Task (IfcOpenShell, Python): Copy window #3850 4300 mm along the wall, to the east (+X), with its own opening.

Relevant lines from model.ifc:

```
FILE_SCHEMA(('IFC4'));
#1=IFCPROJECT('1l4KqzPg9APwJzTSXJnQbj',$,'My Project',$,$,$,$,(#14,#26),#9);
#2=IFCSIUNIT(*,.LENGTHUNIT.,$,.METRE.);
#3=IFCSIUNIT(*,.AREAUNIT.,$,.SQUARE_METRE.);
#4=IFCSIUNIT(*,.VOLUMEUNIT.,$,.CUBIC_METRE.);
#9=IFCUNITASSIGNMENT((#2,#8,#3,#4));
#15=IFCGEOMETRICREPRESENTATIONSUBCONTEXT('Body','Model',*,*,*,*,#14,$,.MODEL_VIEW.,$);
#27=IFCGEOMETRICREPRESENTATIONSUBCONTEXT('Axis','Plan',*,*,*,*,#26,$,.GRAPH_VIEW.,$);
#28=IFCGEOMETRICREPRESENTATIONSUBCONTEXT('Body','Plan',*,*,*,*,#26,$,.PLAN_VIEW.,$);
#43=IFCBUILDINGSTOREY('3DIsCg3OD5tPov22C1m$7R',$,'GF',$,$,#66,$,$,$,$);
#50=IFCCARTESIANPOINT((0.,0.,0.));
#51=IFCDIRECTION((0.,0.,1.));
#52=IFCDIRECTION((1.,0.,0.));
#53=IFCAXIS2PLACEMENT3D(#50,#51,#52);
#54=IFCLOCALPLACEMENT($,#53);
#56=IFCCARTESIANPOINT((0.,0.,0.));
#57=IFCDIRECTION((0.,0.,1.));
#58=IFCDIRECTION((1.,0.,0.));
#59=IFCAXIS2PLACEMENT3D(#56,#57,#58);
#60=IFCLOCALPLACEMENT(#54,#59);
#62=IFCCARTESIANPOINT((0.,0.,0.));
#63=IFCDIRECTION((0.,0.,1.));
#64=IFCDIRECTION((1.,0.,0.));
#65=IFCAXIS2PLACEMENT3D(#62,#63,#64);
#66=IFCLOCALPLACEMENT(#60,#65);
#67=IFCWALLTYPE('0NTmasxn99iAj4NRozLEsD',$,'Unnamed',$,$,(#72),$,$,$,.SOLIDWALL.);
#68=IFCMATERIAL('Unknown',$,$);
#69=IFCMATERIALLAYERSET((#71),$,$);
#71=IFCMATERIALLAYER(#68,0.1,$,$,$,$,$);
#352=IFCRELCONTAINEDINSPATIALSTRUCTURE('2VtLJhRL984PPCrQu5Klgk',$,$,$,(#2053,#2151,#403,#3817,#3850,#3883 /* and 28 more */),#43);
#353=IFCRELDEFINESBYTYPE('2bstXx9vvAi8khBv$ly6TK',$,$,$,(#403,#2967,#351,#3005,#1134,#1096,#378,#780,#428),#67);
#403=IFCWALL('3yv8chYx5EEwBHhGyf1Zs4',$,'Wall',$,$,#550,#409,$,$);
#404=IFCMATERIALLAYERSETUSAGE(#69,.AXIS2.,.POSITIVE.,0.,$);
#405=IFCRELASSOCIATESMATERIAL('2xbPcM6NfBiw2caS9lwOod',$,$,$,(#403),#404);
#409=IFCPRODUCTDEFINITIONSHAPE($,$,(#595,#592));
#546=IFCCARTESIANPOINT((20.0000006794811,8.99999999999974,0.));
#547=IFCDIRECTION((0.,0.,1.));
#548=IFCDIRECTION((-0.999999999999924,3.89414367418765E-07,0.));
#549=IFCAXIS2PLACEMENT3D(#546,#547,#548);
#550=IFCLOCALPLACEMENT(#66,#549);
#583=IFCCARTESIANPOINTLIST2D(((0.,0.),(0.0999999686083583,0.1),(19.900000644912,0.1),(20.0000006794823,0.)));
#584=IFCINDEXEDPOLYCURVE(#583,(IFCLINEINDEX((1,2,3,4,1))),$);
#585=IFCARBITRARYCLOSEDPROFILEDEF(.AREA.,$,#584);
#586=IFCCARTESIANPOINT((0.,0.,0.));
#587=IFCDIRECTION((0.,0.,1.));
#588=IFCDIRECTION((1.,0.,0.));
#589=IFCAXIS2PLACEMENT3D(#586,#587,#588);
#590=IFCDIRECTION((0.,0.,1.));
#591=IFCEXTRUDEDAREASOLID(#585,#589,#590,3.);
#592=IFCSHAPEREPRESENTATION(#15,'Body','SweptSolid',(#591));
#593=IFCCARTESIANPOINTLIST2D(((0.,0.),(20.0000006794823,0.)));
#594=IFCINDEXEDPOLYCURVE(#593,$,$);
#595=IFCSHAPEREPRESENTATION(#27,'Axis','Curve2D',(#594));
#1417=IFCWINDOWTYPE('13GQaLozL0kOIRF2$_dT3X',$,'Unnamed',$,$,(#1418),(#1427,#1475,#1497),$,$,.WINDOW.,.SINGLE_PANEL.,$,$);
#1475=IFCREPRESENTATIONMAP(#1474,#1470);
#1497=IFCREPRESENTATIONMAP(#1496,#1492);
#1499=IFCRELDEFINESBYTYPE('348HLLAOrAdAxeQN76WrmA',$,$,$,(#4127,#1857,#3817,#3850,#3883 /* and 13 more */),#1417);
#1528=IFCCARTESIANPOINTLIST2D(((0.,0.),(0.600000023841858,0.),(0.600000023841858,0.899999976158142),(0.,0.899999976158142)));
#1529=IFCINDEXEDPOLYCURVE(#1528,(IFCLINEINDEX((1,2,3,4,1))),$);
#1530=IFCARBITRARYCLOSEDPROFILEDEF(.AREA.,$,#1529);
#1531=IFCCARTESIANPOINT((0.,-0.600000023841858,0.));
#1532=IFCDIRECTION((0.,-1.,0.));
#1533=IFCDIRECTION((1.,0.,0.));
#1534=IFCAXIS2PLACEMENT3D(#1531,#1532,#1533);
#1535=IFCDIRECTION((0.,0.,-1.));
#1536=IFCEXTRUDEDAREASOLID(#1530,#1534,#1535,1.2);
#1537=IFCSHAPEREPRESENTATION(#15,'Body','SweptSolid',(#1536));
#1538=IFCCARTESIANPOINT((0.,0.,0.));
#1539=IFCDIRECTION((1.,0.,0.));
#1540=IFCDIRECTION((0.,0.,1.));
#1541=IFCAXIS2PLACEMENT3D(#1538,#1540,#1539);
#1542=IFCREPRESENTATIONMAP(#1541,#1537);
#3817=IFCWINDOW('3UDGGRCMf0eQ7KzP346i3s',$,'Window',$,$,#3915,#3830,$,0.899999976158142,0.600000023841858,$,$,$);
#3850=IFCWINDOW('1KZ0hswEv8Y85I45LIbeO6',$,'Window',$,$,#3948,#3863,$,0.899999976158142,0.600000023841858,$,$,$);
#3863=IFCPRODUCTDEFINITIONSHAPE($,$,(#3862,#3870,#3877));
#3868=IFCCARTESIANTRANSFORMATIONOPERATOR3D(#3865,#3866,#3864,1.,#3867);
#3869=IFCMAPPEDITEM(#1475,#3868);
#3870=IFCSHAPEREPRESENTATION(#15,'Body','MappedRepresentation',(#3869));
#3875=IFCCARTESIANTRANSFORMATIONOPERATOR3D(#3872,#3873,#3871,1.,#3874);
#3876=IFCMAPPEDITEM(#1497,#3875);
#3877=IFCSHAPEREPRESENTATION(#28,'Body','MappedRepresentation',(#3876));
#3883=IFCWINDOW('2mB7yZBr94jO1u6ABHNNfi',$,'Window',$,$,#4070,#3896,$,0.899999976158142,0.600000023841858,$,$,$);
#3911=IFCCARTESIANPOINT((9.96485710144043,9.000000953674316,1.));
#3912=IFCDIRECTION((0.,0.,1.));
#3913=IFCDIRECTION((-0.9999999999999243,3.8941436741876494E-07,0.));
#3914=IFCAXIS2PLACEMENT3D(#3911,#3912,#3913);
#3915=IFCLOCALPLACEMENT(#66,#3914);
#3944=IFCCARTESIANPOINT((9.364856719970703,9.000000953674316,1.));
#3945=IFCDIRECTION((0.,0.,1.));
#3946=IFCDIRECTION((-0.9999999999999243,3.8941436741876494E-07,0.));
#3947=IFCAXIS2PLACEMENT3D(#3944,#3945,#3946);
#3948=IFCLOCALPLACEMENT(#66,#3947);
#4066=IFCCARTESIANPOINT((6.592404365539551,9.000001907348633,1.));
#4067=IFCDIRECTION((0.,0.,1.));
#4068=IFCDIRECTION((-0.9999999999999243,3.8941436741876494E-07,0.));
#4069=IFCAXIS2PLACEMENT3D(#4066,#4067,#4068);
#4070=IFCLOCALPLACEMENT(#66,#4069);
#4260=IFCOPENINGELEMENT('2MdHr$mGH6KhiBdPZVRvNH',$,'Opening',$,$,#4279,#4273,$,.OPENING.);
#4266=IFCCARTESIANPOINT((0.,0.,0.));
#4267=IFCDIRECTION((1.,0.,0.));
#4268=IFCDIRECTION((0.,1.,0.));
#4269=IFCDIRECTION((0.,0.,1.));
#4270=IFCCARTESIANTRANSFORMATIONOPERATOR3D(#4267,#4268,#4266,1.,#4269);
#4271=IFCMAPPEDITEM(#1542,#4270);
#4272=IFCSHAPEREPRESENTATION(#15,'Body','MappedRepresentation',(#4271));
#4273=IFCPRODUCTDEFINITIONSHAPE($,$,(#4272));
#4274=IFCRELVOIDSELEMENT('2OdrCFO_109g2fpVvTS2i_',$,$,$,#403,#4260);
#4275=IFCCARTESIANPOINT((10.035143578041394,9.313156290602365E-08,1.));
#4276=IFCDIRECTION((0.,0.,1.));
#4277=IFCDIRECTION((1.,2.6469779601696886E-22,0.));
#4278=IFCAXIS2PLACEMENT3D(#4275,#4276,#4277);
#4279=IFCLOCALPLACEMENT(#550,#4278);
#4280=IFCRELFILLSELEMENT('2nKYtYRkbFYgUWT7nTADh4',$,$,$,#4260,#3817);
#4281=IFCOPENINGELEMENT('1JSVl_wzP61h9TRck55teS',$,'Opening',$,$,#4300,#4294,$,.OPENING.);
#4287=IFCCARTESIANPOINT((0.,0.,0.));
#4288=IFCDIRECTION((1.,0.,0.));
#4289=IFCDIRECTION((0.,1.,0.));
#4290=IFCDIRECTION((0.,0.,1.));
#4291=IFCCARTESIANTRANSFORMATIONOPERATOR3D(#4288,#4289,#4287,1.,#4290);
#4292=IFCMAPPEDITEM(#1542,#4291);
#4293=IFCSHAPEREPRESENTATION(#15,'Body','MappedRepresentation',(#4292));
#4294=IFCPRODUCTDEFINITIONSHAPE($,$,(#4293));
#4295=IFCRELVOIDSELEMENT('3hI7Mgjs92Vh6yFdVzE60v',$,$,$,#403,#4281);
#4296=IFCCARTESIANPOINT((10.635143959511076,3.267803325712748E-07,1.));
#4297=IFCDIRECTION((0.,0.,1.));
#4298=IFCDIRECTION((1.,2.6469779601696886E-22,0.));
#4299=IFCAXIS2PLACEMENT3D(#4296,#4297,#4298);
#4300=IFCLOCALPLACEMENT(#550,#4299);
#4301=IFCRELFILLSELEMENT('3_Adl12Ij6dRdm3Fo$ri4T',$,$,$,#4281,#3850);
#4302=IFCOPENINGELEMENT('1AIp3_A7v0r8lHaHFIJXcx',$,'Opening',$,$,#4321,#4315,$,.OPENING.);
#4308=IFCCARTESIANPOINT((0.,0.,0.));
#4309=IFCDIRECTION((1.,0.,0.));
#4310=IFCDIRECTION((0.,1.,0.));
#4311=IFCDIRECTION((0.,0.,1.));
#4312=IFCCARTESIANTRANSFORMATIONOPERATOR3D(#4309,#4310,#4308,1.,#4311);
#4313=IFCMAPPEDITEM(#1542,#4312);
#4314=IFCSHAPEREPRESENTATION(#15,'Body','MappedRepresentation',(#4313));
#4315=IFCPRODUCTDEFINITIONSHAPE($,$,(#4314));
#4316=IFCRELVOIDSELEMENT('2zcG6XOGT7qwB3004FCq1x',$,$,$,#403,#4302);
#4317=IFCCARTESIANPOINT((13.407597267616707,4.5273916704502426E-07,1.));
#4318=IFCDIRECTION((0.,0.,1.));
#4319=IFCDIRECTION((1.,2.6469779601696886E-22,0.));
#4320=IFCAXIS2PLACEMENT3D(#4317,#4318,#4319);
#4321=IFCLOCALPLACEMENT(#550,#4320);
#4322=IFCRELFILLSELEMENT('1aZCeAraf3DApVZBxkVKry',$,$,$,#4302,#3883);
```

```python
import ifcopenshell
import ifcopenshell.api.feature
import ifcopenshell.api.geometry
import ifcopenshell.api.root
import ifcopenshell.geom
import ifcopenshell.util.element
import ifcopenshell.util.placement
import ifcopenshell.util.shape
import ifcopenshell.util.unit

model = ifcopenshell.open("model.ifc")
unit_scale = ifcopenshell.util.unit.calculate_unit_scale(model)
settings = ifcopenshell.geom.settings()


def volume(element):
    """Net volume in cubic metres, openings subtracted."""
    shape = ifcopenshell.geom.create_shape(settings, element)
    return ifcopenshell.util.shape.get_volume(shape.geometry)


window = model.by_id(3850)
opening = window.FillsVoids[0].RelatingOpeningElement
wall = opening.VoidsElements[0].RelatingBuildingElement
before = volume(wall)
shift = ifcopenshell.util.placement.get_local_placement(wall.ObjectPlacement)[:3, 0] * -4.3 / unit_scale

# copy_class copies the void relationship, type, container and properties, but no geometry.
new_opening = ifcopenshell.api.root.copy_class(model, product=opening)
new_opening.Representation = ifcopenshell.util.element.copy_deep(
    model, opening.Representation, exclude=["IfcGeometricRepresentationContext", "IfcRepresentationMap"]
)
new_window = ifcopenshell.api.root.copy_class(model, product=window)
new_window.Representation = ifcopenshell.util.element.copy_deep(
    model, window.Representation, exclude=["IfcGeometricRepresentationContext", "IfcRepresentationMap"]
)
ifcopenshell.api.feature.add_filling(model, opening=new_opening, element=new_window)

for old, new in ((opening, new_opening), (window, new_window)):
    matrix = ifcopenshell.util.placement.get_local_placement(old.ObjectPlacement)
    matrix[:3, 3] += shift
    ifcopenshell.api.geometry.edit_object_placement(model, product=new, matrix=matrix, is_si=False)

after = volume(wall)

print(f"wall volume {before:.3f} -> {after:.3f} m3")

model.write("model_rev.ifc")
```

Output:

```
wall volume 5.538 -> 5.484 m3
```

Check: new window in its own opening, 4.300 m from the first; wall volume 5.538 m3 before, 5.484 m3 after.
